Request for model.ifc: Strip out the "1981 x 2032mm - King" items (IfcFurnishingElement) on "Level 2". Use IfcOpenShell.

First a look at what the model holds.

```python
import ifcopenshell
import ifcopenshell.util.element

model = ifcopenshell.open("model.ifc")
print(model.schema)
storey = next(s for s in model.by_type("IfcBuildingStorey") if s.Name == "Level 2")
furniture = [e for e in ifcopenshell.util.element.get_decomposition(storey) if e.is_a("IfcFurnishingElement")]
seen = {}
for e in furniture:
    element_type = ifcopenshell.util.element.get_type(e)
    name = element_type.Name if element_type not in (None, e) else None
    seen[name] = seen.get(name, 0) + 1
for name, count in sorted(seen.items(), key=str):
    print(count, "x", name)
```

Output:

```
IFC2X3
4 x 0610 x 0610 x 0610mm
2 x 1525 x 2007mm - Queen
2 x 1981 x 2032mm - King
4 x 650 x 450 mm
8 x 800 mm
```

```python
import ifcopenshell
import ifcopenshell.api.root
import ifcopenshell.util.element

model = ifcopenshell.open("model.ifc")

storey = next(s for s in model.by_type("IfcBuildingStorey") if s.Name == "Level 2")
furniture = [e for e in ifcopenshell.util.element.get_decomposition(storey) if e.is_a("IfcFurnishingElement")]
targets = [e for e in furniture if (t := ifcopenshell.util.element.get_type(e)) not in (None, e) and t.Name == "1981 x 2032mm - King"]

for e in targets:
    ifcopenshell.api.root.remove_product(model, product=e)
print(len(targets), "removed")

model.write("model_rev.ifc")
```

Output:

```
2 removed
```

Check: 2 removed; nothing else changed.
